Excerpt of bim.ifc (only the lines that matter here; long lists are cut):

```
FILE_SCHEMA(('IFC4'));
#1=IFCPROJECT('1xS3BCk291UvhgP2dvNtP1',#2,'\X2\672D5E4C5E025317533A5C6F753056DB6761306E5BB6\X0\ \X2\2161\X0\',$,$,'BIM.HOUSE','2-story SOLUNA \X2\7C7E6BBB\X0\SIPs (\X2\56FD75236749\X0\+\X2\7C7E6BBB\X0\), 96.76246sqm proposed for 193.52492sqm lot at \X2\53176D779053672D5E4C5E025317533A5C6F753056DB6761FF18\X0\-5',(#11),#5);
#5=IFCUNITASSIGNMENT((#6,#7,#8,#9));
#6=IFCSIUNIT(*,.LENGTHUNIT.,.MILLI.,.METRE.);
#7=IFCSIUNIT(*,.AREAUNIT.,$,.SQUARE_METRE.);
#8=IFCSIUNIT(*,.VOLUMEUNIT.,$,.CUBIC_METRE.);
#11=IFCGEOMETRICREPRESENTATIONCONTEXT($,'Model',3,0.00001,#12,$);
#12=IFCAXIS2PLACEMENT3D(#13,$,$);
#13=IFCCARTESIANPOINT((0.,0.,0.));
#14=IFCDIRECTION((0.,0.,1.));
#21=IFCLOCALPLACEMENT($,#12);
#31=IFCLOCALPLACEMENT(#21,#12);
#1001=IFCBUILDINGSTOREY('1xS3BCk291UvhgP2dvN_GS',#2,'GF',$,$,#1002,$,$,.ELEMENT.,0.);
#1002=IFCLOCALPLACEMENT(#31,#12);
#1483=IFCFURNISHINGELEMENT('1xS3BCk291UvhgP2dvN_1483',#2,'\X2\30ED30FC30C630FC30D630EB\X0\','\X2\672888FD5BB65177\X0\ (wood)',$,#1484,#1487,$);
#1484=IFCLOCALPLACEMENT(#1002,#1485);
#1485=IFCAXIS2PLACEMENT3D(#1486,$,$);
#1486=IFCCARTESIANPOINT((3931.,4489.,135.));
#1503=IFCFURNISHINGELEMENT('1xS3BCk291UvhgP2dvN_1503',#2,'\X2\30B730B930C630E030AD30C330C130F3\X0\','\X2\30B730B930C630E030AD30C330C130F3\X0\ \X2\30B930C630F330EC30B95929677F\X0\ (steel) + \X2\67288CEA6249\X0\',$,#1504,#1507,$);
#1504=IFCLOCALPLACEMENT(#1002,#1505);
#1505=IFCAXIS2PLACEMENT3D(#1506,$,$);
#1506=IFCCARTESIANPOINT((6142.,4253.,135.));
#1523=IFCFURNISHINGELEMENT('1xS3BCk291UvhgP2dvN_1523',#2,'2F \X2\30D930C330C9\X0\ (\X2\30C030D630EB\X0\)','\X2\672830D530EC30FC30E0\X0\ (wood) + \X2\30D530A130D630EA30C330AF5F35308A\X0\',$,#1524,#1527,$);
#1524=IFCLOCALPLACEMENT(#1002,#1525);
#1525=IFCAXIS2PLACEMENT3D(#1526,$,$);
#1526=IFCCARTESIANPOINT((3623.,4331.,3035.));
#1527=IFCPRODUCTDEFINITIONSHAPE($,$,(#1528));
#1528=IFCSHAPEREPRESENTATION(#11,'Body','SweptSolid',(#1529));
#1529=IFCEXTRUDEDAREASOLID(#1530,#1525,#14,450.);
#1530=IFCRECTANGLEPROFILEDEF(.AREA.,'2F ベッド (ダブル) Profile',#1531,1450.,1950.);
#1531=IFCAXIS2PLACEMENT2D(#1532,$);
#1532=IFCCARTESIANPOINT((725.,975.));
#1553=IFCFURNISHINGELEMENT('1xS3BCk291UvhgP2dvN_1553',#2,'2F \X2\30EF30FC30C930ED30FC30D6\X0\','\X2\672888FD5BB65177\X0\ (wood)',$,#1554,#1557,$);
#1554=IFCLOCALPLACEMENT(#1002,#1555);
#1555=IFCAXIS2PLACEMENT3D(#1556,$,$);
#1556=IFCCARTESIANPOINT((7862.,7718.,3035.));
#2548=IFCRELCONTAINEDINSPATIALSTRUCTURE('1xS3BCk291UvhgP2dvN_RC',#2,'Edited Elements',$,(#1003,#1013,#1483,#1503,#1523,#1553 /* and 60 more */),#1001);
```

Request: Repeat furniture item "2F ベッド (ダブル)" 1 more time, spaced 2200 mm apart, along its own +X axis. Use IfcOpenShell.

```python
import ifcopenshell
import ifcopenshell.api.geometry
import ifcopenshell.api.root
import ifcopenshell.util.element
import ifcopenshell.util.placement

model = ifcopenshell.open("bim.ifc")


def reuse_history(source, copy):
    """copy_class also copies each property set's owner history, people and application; keep the originals."""
    for rel in copy.IsDefinedBy:
        if rel.is_a("IfcRelDefinesByProperties") and (history := rel.RelatingPropertyDefinition.OwnerHistory):
            rel.RelatingPropertyDefinition.OwnerHistory = source.OwnerHistory
            ifcopenshell.util.element.remove_deep2(model, history)


source = model.by_guid("1xS3BCk291UvhgP2dvN_1523")
base = ifcopenshell.util.placement.get_local_placement(source.ObjectPlacement)
step = base[:3, 0] * 2200.0

for i in range(1, 2):
    copy = ifcopenshell.api.root.copy_class(model, product=source)
    copy.Representation = ifcopenshell.util.element.copy_deep(
        model, source.Representation, exclude=["IfcGeometricRepresentationContext", "IfcRepresentationMap"]
    )
    reuse_history(source, copy)
    matrix = base.copy()
    matrix[:3, 3] += i * step
    print("added at", matrix[:3, 3].round(3) + 0.0)
    ifcopenshell.api.geometry.edit_object_placement(model, product=copy, matrix=matrix, is_si=False)

model.write("bim_updated.ifc")
```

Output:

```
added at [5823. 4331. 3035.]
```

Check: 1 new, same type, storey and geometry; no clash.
